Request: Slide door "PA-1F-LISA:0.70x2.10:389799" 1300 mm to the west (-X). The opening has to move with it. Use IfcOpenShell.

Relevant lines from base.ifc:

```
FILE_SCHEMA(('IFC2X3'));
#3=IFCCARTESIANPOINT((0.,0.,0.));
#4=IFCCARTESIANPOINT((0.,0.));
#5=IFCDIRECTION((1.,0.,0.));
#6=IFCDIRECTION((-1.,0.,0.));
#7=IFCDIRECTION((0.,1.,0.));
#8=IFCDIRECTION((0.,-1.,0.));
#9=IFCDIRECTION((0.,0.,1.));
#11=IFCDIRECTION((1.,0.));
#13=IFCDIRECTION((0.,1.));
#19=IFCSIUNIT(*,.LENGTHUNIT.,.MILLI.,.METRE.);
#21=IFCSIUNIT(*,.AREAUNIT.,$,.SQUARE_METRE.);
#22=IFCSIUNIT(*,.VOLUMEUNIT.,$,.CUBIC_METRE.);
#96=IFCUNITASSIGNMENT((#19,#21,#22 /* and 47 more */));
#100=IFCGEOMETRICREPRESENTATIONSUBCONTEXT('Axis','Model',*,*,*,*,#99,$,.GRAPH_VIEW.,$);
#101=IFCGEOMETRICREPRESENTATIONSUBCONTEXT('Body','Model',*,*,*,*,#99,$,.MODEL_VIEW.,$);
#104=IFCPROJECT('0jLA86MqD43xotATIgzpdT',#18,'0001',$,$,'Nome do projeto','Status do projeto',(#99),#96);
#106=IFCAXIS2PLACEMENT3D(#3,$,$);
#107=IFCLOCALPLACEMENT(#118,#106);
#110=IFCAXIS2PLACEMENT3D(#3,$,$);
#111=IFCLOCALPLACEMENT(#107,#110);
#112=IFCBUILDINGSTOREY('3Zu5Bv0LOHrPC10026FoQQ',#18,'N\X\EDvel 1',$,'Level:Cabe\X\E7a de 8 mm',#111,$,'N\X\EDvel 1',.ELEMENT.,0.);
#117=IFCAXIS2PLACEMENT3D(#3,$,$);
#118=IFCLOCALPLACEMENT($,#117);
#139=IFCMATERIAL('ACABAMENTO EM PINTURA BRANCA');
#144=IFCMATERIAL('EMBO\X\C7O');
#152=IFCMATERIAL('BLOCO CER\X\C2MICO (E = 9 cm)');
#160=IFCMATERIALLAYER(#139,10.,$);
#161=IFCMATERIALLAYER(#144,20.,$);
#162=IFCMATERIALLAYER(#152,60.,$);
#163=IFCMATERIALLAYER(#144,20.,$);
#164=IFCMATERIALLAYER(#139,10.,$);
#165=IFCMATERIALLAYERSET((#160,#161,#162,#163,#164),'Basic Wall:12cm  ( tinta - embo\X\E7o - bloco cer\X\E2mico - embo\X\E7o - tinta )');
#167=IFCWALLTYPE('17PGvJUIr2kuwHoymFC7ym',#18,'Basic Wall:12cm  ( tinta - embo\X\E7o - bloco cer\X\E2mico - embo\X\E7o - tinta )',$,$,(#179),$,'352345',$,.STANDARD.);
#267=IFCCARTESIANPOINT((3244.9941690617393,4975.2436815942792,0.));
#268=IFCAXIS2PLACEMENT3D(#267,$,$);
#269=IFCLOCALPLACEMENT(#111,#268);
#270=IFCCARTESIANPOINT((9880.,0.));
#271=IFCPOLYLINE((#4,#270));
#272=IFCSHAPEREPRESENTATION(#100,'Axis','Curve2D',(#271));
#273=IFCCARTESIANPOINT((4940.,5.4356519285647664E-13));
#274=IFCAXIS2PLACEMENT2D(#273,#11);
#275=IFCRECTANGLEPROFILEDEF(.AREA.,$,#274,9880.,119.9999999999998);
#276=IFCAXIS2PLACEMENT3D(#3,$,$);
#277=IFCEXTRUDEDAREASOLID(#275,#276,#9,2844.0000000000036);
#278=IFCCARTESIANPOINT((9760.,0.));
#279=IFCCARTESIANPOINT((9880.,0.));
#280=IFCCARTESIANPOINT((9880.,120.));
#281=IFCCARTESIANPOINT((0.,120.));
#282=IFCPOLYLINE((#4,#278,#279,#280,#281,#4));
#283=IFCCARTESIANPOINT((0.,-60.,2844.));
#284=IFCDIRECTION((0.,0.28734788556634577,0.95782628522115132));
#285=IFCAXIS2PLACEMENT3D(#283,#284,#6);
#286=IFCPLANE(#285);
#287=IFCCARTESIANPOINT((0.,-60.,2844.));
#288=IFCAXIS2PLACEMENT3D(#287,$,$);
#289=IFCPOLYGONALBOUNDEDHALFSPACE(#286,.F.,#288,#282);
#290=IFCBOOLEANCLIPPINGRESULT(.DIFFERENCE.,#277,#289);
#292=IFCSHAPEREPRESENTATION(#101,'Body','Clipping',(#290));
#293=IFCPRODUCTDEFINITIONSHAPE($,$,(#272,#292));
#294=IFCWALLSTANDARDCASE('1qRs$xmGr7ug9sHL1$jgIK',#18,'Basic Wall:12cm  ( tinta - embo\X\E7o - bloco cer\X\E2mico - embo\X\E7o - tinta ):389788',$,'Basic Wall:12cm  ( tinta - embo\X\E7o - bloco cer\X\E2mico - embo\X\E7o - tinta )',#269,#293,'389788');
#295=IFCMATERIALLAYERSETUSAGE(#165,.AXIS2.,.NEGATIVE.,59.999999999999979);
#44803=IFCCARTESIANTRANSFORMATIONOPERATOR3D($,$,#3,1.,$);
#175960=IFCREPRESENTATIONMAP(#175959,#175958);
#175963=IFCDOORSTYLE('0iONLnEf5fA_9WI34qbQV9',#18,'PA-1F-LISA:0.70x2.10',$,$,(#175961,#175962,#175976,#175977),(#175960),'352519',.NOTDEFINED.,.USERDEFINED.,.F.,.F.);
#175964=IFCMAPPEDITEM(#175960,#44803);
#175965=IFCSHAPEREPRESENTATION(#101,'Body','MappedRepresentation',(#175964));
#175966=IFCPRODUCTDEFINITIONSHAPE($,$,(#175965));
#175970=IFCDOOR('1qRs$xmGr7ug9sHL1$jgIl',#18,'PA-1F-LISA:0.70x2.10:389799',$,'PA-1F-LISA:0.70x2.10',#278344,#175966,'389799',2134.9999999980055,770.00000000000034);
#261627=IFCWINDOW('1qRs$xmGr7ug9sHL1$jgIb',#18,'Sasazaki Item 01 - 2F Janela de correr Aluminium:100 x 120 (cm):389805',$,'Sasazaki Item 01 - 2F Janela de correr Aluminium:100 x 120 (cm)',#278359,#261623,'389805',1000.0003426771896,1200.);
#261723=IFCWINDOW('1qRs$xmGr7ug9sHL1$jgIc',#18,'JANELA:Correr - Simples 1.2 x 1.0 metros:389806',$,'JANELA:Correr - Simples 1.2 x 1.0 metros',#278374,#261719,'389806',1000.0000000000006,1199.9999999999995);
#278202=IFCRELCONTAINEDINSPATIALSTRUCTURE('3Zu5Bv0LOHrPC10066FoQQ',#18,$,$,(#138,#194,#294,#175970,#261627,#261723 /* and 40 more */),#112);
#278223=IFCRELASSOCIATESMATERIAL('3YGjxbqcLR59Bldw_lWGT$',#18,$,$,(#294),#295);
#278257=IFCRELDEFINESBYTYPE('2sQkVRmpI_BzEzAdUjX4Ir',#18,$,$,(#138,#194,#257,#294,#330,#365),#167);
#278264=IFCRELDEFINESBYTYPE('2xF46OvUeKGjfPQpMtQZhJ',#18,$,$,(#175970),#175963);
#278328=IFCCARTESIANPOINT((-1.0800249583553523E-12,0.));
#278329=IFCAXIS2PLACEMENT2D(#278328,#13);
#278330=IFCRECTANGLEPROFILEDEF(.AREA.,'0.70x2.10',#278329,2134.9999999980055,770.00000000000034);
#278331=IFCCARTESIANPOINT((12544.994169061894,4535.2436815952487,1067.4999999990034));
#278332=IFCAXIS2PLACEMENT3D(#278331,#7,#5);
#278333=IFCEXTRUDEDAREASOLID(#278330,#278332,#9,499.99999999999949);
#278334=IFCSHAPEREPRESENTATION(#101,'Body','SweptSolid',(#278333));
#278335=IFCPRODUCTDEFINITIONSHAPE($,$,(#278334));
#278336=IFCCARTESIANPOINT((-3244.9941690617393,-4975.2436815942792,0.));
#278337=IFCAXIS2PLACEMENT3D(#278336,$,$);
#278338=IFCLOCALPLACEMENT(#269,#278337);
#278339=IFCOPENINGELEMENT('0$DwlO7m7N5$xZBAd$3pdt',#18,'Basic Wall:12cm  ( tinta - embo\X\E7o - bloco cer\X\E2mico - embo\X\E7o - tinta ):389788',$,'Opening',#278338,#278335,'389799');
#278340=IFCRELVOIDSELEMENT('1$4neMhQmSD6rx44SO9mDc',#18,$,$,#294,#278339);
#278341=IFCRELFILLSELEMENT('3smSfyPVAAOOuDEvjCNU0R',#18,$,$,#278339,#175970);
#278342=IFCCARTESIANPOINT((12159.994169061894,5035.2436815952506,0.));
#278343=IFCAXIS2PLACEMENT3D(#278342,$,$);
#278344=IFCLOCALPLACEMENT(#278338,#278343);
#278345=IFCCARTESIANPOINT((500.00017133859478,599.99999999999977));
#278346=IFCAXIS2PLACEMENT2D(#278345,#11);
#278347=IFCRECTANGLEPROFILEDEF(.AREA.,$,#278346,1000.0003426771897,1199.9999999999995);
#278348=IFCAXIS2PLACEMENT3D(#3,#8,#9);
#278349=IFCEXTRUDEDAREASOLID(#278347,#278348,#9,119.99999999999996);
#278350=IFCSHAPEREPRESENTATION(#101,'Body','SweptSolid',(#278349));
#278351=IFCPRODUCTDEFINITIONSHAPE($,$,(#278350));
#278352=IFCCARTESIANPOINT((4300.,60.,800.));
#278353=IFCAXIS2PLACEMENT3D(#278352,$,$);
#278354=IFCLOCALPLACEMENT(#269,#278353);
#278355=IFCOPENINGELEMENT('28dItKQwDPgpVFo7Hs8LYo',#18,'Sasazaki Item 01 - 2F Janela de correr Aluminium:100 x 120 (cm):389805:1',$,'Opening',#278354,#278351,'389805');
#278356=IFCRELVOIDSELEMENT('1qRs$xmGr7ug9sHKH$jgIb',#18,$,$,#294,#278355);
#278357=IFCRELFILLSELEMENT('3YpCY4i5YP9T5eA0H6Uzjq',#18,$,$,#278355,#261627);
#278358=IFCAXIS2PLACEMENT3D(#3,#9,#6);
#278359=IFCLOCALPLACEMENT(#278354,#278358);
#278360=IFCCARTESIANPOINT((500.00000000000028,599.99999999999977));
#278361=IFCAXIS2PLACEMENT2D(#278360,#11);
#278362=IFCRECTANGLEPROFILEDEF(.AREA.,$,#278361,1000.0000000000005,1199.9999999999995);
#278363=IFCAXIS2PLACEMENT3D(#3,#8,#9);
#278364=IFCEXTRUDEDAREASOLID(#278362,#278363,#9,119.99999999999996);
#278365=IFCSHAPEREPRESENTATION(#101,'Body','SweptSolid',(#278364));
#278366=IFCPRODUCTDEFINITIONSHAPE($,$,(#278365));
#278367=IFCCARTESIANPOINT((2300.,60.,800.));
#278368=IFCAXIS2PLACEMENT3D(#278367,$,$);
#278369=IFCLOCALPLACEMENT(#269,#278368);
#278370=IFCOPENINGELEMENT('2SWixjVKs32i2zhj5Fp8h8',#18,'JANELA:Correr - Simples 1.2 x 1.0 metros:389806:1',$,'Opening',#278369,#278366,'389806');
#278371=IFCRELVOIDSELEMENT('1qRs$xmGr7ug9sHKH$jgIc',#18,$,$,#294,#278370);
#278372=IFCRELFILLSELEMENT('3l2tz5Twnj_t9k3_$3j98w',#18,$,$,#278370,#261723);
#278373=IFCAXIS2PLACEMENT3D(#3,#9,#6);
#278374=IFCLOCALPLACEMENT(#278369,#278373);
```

```python
import ifcopenshell
import ifcopenshell.api.geometry
import ifcopenshell.util.placement

model = ifcopenshell.open("base.ifc")

door = model.by_guid("1qRs$xmGr7ug9sHL1$jgIl")
opening = door.FillsVoids[0].RelatingOpeningElement
wall = opening.VoidsElements[0].RelatingBuildingElement

wall_matrix = ifcopenshell.util.placement.get_local_placement(wall.ObjectPlacement)
shift = wall_matrix[:3, 0] * -1300.0
before = ifcopenshell.util.placement.get_local_placement(door.ObjectPlacement)[:3, 3].copy()

# The door is placed relative to its opening, so it follows when the opening moves.
matrix = ifcopenshell.util.placement.get_local_placement(opening.ObjectPlacement)
matrix[:3, 3] += shift
ifcopenshell.api.geometry.edit_object_placement(
    model, product=opening, matrix=matrix, is_si=False, should_transform_children=True
)

after = ifcopenshell.util.placement.get_local_placement(door.ObjectPlacement)[:3, 3]
print("door moved by", (after - before).round(3) + 0.0)

model.write("base_v2.ifc")
```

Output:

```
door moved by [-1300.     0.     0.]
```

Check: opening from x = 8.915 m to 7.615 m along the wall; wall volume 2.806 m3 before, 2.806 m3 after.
